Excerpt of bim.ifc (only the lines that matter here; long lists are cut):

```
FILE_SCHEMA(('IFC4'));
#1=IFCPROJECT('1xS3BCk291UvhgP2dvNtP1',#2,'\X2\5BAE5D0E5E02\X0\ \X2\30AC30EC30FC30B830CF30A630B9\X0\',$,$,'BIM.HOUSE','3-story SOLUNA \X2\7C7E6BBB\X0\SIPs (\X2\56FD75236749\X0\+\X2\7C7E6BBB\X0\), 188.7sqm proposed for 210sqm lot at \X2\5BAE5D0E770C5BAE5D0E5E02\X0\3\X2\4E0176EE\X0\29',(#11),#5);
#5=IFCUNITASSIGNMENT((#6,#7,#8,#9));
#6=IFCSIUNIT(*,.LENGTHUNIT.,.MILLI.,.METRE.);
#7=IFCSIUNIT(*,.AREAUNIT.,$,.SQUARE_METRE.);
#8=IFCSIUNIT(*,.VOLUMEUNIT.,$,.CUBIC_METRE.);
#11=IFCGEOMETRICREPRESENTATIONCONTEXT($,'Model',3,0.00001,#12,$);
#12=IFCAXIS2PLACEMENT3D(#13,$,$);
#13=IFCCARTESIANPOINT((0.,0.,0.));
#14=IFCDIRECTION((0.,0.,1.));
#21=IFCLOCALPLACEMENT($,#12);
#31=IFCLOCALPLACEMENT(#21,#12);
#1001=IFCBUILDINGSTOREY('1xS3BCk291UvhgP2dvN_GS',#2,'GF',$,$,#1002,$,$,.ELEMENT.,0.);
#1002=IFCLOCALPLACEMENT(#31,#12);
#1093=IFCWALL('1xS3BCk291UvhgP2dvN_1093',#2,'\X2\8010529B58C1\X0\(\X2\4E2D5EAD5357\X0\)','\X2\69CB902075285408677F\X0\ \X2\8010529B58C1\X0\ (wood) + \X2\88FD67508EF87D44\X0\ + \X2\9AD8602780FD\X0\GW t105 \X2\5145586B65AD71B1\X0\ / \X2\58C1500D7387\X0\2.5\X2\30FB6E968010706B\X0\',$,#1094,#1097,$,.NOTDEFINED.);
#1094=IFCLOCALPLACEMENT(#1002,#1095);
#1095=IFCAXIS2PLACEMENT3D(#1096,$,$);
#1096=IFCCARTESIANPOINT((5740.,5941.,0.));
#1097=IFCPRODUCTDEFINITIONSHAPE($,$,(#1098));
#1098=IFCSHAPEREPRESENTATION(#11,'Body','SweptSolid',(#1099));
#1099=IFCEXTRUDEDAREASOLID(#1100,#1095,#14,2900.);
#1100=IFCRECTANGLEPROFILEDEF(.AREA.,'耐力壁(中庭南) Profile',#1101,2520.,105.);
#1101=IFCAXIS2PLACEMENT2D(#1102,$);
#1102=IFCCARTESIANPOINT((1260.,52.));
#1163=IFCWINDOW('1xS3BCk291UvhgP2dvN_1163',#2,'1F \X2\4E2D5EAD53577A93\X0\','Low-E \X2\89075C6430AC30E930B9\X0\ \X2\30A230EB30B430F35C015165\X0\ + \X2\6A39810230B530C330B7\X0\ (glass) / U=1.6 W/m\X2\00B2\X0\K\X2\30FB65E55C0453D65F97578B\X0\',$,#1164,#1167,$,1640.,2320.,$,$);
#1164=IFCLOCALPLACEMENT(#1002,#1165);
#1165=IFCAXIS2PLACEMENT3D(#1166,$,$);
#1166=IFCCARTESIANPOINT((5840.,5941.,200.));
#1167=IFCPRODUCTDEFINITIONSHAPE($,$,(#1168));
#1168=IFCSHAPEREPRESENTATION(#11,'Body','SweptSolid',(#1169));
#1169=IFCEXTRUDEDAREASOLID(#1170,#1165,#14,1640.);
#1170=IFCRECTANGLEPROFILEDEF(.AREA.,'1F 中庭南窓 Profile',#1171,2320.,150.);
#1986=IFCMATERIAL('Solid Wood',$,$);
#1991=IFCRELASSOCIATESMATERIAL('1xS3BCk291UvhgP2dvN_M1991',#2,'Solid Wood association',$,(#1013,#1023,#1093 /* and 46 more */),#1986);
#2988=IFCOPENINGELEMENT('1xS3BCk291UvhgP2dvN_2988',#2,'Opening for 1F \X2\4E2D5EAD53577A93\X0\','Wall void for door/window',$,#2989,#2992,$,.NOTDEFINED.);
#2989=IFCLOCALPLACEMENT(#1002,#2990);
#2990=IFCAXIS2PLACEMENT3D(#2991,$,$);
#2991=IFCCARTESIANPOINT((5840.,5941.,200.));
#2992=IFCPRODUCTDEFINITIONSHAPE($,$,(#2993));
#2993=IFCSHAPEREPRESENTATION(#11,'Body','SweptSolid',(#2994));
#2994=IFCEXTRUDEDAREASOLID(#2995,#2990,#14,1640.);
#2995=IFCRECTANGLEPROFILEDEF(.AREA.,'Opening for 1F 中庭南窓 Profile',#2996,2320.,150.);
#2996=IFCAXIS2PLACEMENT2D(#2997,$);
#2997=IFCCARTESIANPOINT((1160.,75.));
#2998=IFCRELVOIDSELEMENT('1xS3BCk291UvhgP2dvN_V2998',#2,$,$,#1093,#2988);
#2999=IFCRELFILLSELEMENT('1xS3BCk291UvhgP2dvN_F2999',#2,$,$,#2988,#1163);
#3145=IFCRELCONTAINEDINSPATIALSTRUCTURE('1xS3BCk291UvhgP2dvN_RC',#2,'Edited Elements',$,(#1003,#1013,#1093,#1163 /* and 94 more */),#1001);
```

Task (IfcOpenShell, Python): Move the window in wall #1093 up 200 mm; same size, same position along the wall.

```python
import numpy as np
import ifcopenshell
import ifcopenshell.api.geometry
import ifcopenshell.util.placement
import ifcopenshell.util.unit

model = ifcopenshell.open("bim.ifc")
unit_scale = ifcopenshell.util.unit.calculate_unit_scale(model)

window = model.by_guid("1xS3BCk291UvhgP2dvN_1163")
opening = window.FillsVoids[0].RelatingOpeningElement
dz = 200.0

shift = np.array([0.0, 0.0, dz])
# The window is not placed relative to its opening, so move both.
for product in (opening, window):
    matrix = ifcopenshell.util.placement.get_local_placement(product.ObjectPlacement)
    matrix[:3, 3] += shift
    ifcopenshell.api.geometry.edit_object_placement(model, product=product, matrix=matrix, is_si=False)

print(f"moved by {dz * unit_scale:+.3f} m")

model.write("bim_v2.ifc")
```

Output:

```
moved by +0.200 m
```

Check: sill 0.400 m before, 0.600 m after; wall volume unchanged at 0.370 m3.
